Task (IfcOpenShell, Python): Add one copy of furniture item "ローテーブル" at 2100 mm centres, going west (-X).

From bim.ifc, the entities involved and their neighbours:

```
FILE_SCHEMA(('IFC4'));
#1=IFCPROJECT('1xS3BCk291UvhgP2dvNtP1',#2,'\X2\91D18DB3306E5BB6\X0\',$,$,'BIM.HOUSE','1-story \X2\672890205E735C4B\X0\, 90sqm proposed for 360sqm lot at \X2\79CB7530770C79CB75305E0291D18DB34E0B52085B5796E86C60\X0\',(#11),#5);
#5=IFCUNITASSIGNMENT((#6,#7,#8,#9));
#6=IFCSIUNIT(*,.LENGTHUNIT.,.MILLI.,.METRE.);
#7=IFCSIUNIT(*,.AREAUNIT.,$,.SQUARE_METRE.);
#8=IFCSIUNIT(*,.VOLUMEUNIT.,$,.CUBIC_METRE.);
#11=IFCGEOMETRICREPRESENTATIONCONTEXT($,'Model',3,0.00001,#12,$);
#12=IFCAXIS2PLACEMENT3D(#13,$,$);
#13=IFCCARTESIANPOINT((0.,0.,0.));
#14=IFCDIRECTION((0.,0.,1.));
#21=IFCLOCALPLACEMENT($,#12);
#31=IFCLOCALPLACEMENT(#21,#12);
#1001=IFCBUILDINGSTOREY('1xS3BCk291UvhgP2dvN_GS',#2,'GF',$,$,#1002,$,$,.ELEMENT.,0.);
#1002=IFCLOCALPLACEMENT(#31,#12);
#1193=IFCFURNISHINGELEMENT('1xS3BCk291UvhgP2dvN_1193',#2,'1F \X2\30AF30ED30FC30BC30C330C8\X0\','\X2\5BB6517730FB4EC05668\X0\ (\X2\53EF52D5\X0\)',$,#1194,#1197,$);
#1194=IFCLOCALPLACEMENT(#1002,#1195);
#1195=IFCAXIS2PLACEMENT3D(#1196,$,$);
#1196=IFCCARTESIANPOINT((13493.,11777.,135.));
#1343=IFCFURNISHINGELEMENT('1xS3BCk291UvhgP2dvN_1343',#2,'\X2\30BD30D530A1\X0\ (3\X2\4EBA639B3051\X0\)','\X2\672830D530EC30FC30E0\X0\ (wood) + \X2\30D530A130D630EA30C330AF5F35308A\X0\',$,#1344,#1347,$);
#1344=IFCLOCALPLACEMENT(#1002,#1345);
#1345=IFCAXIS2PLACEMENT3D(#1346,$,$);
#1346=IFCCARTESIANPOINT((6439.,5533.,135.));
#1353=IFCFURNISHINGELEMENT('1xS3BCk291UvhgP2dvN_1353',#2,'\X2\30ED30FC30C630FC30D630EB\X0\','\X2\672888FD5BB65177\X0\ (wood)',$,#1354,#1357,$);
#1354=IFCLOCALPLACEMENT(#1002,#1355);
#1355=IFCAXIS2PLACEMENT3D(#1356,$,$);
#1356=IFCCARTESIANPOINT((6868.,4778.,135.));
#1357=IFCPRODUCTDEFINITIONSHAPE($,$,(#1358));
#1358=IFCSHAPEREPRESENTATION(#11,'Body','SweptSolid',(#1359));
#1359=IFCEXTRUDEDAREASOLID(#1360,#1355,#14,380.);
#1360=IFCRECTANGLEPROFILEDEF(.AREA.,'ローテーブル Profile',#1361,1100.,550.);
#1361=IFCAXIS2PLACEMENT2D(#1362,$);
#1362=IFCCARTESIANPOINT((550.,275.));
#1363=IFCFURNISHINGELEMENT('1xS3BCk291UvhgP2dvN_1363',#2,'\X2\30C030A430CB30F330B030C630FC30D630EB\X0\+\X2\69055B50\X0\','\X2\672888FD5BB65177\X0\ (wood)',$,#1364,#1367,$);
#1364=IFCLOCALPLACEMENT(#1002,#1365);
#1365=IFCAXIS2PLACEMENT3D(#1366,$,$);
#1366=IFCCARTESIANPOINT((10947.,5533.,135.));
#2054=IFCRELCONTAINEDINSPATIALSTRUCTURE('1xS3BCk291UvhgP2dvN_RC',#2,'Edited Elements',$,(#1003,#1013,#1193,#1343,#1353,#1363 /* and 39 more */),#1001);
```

```python
import numpy as np
import ifcopenshell
import ifcopenshell.api.geometry
import ifcopenshell.api.root
import ifcopenshell.util.element
import ifcopenshell.util.placement
import ifcopenshell.util.unit

model = ifcopenshell.open("bim.ifc")
unit_scale = ifcopenshell.util.unit.calculate_unit_scale(model)


def reuse_history(source, copy):
    """copy_class also copies each property set's owner history, people and application; keep the originals."""
    for rel in copy.IsDefinedBy:
        if rel.is_a("IfcRelDefinesByProperties") and (history := rel.RelatingPropertyDefinition.OwnerHistory):
            rel.RelatingPropertyDefinition.OwnerHistory = source.OwnerHistory
            ifcopenshell.util.element.remove_deep2(model, history)


source = model.by_guid("1xS3BCk291UvhgP2dvN_1353")
base = ifcopenshell.util.placement.get_local_placement(source.ObjectPlacement)
step = np.array([-1.0, 0.0, 0.0]) * 2.1 / unit_scale

for i in range(1, 2):
    copy = ifcopenshell.api.root.copy_class(model, product=source)
    copy.Representation = ifcopenshell.util.element.copy_deep(
        model, source.Representation, exclude=["IfcGeometricRepresentationContext", "IfcRepresentationMap"]
    )
    reuse_history(source, copy)
    matrix = base.copy()
    matrix[:3, 3] += i * step
    print("added at", matrix[:3, 3].round(3) + 0.0)
    ifcopenshell.api.geometry.edit_object_placement(model, product=copy, matrix=matrix, is_si=False)

model.write("bim_edited.ifc")
```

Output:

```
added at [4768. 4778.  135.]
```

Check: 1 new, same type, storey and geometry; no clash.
